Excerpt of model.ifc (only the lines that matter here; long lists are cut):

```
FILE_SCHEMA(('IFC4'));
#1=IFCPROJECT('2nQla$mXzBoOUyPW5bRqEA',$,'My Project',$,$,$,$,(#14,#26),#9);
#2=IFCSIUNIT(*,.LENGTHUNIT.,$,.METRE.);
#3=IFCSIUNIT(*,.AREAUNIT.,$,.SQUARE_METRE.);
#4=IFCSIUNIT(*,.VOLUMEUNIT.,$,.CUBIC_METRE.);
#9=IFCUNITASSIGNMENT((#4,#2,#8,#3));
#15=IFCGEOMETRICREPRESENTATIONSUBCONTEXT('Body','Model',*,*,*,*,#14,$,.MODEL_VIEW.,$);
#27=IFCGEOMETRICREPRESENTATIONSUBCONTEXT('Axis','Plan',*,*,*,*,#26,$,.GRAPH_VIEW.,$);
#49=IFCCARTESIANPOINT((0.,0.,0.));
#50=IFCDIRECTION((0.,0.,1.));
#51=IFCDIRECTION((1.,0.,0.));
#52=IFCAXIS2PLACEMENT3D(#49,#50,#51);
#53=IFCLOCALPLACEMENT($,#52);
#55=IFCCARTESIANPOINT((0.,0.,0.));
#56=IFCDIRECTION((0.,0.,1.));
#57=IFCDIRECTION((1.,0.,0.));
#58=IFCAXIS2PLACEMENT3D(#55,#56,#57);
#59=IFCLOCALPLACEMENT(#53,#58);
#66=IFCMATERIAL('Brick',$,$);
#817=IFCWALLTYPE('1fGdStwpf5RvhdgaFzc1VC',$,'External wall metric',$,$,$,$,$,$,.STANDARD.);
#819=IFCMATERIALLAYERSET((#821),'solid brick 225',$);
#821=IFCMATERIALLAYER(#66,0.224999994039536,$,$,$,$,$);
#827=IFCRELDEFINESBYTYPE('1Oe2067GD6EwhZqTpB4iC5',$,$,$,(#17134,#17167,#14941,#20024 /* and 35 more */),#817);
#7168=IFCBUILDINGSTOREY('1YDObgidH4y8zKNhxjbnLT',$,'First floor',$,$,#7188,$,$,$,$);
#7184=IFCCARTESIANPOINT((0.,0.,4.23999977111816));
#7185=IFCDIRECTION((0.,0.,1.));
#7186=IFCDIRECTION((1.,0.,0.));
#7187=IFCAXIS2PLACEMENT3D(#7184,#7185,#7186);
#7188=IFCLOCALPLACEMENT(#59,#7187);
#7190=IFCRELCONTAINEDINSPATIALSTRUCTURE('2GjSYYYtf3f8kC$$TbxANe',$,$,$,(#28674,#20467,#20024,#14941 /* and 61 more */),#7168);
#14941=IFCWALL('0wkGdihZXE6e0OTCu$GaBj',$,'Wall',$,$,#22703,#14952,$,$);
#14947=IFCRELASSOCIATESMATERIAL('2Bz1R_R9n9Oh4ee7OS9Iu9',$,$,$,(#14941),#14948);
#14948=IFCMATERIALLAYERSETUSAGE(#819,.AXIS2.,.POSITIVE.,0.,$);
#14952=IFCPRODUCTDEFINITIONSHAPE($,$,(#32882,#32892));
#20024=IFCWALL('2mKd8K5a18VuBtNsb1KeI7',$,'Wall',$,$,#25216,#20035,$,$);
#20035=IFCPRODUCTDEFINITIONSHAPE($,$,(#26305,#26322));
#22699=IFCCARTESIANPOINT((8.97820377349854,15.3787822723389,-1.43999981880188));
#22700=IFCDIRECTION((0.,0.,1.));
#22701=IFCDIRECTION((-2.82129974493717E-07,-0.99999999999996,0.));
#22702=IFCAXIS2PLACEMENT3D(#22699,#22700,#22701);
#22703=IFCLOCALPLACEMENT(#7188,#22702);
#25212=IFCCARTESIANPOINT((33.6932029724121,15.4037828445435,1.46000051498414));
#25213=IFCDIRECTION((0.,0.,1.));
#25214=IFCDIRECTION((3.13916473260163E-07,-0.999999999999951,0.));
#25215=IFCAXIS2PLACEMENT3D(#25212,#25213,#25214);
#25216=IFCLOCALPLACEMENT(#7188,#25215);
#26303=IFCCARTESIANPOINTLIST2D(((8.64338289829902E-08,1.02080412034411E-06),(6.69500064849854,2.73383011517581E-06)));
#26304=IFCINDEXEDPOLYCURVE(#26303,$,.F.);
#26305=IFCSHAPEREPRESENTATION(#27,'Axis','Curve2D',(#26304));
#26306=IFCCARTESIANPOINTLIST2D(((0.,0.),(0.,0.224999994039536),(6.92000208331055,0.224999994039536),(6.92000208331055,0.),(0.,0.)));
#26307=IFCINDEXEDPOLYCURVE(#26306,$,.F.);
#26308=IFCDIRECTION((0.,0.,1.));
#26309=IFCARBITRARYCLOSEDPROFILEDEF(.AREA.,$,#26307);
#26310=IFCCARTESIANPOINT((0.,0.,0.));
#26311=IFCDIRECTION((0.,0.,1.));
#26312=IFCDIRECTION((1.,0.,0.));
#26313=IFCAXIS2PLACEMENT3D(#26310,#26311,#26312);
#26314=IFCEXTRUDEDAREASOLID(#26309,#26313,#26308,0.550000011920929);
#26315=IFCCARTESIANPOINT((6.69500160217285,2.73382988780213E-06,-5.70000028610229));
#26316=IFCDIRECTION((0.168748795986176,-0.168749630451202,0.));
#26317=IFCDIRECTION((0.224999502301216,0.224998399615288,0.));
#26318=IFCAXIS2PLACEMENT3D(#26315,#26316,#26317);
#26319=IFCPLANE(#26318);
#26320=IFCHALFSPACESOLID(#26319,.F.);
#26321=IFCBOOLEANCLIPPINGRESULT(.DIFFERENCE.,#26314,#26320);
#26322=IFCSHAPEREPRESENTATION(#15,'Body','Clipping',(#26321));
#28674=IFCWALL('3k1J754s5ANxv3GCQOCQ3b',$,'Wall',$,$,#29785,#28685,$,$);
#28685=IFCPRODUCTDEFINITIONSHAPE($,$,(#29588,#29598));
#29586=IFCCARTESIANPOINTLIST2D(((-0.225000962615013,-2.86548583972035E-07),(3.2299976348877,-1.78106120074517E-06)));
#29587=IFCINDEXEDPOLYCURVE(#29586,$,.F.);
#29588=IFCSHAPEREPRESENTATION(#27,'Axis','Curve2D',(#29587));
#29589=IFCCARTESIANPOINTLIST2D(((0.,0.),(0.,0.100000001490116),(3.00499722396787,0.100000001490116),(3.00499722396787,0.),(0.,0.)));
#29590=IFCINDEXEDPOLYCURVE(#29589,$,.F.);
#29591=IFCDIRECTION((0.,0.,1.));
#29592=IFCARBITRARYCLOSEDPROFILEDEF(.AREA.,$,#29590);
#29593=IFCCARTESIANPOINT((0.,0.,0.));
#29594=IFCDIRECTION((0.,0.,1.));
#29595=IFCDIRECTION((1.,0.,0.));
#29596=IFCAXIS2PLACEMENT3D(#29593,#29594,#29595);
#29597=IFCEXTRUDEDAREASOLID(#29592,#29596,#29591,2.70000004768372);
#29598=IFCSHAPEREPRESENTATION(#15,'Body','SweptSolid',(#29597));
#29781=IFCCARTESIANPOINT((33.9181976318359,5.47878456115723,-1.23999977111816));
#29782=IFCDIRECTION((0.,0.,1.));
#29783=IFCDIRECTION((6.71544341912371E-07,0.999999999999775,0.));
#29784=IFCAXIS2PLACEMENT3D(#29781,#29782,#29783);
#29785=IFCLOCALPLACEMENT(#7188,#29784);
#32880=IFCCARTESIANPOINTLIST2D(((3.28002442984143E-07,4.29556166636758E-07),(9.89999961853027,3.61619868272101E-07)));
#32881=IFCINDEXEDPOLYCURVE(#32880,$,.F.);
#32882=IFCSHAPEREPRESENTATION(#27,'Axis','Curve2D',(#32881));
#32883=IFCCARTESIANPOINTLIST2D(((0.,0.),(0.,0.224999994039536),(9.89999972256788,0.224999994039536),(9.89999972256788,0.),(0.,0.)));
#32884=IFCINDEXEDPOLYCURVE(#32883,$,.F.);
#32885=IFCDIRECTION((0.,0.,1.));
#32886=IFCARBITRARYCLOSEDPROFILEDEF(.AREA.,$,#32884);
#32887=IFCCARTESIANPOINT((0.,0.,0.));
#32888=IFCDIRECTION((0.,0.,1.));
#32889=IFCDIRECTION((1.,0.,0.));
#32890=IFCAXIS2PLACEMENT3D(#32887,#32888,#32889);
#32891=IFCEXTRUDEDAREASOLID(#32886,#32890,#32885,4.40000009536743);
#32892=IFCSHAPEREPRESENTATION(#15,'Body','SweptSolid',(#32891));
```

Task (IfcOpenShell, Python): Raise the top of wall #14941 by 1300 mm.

```python
import ifcopenshell
import ifcopenshell.geom
import ifcopenshell.util.representation
import ifcopenshell.util.shape

model = ifcopenshell.open("model.ifc")
settings = ifcopenshell.geom.settings()


def volume(element):
    """Net volume in cubic metres, openings subtracted."""
    shape = ifcopenshell.geom.create_shape(settings, element)
    return ifcopenshell.util.shape.get_volume(shape.geometry)


wall = model.by_guid("0wkGdihZXE6e0OTCu$GaBj")
before = volume(wall)

body = ifcopenshell.util.representation.get_representation(wall, "Model", "Body")
solid = body.Items[0]
old_height = solid.Depth
solid.Depth += 1.3
after = volume(wall)

print(f"height {old_height:g} -> {solid.Depth:g}, volume {before:.3f} -> {after:.3f} m3")

model.write("model_rev.ifc")
```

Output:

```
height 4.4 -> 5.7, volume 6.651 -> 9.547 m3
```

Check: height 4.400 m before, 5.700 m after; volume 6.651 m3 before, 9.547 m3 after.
